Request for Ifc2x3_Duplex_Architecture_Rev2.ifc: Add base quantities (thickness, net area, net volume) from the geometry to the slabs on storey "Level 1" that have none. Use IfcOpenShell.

First a look at what the model holds.

```python
import ifcopenshell
import ifcopenshell.util.element
import ifcopenshell.util.unit

model = ifcopenshell.open("Ifc2x3_Duplex_Architecture_Rev2.ifc")
print(model.schema)
for unit_type in ("LENGTHUNIT", "AREAUNIT", "VOLUMEUNIT"):
    print(unit_type, ifcopenshell.util.unit.calculate_unit_scale(model, unit_type))
storey = next(s for s in model.by_type("IfcBuildingStorey") if s.Name == "Level 1")
slabs = [e for e in ifcopenshell.util.element.get_decomposition(storey) if e.is_a("IfcSlab")]
for e in sorted(slabs, key=lambda e: e.id()):
    print(e.id(), e.is_a(), e.Name, list(ifcopenshell.util.element.get_psets(e, qtos_only=True)), sep=" | ")
```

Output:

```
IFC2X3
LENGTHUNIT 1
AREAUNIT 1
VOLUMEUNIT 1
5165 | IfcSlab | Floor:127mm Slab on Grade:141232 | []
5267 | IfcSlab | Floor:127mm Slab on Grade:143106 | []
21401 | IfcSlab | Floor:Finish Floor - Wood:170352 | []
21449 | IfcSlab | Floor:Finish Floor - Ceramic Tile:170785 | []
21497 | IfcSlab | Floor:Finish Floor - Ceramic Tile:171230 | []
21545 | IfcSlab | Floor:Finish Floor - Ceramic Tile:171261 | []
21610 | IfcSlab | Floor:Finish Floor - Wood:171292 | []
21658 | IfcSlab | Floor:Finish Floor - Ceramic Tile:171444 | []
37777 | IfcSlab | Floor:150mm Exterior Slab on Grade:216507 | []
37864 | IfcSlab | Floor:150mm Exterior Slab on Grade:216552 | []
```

```python
import ifcopenshell
import ifcopenshell.api.pset
import ifcopenshell.geom
import ifcopenshell.util.element
import ifcopenshell.util.shape
import ifcopenshell.util.unit

model = ifcopenshell.open("Ifc2x3_Duplex_Architecture_Rev2.ifc")
unit_scale = ifcopenshell.util.unit.calculate_unit_scale(model)
area_scale = ifcopenshell.util.unit.calculate_unit_scale(model, "AREAUNIT")
volume_scale = ifcopenshell.util.unit.calculate_unit_scale(model, "VOLUMEUNIT")
settings = ifcopenshell.geom.settings()

storey = next(s for s in model.by_type("IfcBuildingStorey") if s.Name == "Level 1")
slabs = [e for e in ifcopenshell.util.element.get_decomposition(storey) if e.is_a("IfcSlab")]

for e in sorted(slabs, key=lambda e: e.id()):
    if ifcopenshell.util.element.get_psets(e, qtos_only=True, should_inherit=False):
        continue
    # Geometry comes back in metres, in the element's own axes.
    shape = ifcopenshell.geom.create_shape(settings, e)
    values = {
        "Width": ifcopenshell.util.shape.get_z(shape.geometry) / unit_scale,
        "NetArea": ifcopenshell.util.shape.get_footprint_area(shape.geometry) / area_scale,
        "NetVolume": ifcopenshell.util.shape.get_volume(shape.geometry) / volume_scale,
    }
    qto = ifcopenshell.api.pset.add_qto(model, product=e, name="BaseQuantities")
    ifcopenshell.api.pset.edit_qto(model, qto=qto, properties=values)
    print(e.id(), {k: round(v, 3) for k, v in values.items()})

model.write("Ifc2x3_Duplex_Architecture_Rev2_v2.ifc")
```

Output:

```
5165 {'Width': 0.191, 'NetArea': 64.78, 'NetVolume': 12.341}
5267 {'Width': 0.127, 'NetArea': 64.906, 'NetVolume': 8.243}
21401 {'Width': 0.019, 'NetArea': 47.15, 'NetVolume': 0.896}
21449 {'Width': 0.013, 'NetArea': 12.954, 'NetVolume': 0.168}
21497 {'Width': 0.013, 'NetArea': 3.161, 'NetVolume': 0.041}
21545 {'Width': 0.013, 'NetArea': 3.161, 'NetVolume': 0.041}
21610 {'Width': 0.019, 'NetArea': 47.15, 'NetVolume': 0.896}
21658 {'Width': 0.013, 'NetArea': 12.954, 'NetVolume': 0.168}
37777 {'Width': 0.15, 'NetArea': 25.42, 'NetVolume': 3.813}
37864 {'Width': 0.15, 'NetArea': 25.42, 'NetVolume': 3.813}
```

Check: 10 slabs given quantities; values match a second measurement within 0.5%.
